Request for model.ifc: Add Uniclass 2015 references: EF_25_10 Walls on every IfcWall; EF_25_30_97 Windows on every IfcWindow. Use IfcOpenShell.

First a look at what the model holds.

```python
import ifcopenshell

model = ifcopenshell.open("model.ifc")
print(model.schema)
print("classifications:", [c.Name for c in model.by_type("IfcClassification")])
for ifc_class in ("IfcDoor", "IfcRoof", "IfcStair", "IfcWall", "IfcWindow"):
    print(ifc_class, len(model.by_type(ifc_class)))
```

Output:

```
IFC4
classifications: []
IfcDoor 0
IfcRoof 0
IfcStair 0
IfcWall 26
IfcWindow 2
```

```python
import ifcopenshell
import ifcopenshell.api.classification

model = ifcopenshell.open("model.ifc")

system = ifcopenshell.api.classification.add_classification(model, classification="Uniclass 2015")

codes = {
    "IfcWall": ("EF_25_10", "Walls"),
    "IfcWindow": ("EF_25_30_97", "Windows"),
}
for ifc_class, (code, name) in codes.items():
    products = model.by_type(ifc_class)
    ifcopenshell.api.classification.add_reference(
        model, products=products, classification=system, identification=code, name=name
    )
    print(code, len(products))

model.write("model_edited.ifc")
```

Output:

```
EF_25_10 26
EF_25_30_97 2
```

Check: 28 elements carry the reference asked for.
